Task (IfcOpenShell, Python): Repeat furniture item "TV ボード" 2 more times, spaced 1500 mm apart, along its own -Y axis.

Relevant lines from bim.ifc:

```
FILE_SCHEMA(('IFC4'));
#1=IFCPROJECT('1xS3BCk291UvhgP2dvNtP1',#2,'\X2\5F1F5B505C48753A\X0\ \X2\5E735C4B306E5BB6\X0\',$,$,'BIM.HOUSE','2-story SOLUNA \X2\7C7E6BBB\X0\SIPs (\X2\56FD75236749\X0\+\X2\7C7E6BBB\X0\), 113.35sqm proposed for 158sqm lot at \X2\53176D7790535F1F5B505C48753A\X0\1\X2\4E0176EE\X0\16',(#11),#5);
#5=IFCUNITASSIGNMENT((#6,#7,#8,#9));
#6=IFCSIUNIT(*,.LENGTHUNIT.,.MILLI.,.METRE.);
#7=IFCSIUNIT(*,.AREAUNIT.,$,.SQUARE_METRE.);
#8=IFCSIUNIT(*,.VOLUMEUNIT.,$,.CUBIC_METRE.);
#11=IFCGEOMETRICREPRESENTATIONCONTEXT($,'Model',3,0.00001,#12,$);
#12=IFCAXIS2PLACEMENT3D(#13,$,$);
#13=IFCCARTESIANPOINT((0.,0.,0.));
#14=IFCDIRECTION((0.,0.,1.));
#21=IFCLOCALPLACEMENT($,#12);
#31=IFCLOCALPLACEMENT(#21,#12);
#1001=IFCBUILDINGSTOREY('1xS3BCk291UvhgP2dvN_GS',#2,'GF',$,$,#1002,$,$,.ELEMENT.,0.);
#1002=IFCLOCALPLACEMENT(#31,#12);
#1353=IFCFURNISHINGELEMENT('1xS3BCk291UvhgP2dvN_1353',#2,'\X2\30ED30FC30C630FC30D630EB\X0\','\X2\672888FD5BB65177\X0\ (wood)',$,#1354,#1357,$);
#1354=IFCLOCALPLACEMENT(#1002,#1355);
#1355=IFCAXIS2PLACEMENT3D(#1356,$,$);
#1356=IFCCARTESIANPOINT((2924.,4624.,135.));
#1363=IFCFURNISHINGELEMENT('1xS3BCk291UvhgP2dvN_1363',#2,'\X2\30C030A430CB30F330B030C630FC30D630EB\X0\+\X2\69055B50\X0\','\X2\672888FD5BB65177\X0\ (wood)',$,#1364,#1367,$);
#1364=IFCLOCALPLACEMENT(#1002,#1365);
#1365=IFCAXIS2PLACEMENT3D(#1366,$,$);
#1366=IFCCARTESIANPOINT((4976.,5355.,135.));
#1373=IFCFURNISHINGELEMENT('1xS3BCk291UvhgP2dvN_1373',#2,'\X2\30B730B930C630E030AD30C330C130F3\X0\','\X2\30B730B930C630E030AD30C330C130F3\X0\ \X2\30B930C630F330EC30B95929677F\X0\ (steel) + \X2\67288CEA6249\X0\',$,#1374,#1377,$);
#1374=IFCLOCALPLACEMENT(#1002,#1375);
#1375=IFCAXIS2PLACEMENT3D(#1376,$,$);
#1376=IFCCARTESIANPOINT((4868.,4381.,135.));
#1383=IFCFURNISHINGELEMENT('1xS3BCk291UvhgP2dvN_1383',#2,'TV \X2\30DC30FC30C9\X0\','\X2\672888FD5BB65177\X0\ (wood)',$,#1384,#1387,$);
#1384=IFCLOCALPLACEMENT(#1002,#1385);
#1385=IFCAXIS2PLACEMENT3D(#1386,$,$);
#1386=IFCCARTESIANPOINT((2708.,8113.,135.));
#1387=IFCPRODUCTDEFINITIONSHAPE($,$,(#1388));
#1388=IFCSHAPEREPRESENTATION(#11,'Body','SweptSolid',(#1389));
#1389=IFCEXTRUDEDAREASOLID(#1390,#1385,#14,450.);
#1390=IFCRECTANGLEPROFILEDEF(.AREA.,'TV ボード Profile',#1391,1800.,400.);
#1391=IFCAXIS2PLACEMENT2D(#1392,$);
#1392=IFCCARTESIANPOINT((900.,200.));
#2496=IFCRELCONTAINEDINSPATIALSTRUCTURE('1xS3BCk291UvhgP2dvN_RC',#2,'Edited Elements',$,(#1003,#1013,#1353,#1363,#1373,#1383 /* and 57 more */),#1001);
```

```python
import ifcopenshell
import ifcopenshell.api.geometry
import ifcopenshell.api.root
import ifcopenshell.util.element
import ifcopenshell.util.placement

model = ifcopenshell.open("bim.ifc")


def reuse_history(source, copy):
    """copy_class also copies each property set's owner history, people and application; keep the originals."""
    for rel in copy.IsDefinedBy:
        if rel.is_a("IfcRelDefinesByProperties") and (history := rel.RelatingPropertyDefinition.OwnerHistory):
            rel.RelatingPropertyDefinition.OwnerHistory = source.OwnerHistory
            ifcopenshell.util.element.remove_deep2(model, history)


source = model.by_guid("1xS3BCk291UvhgP2dvN_1383")
base = ifcopenshell.util.placement.get_local_placement(source.ObjectPlacement)
step = -base[:3, 1] * 1500.0

for i in range(1, 3):
    copy = ifcopenshell.api.root.copy_class(model, product=source)
    copy.Representation = ifcopenshell.util.element.copy_deep(
        model, source.Representation, exclude=["IfcGeometricRepresentationContext", "IfcRepresentationMap"]
    )
    reuse_history(source, copy)
    matrix = base.copy()
    matrix[:3, 3] += i * step
    print("added at", matrix[:3, 3].round(3) + 0.0)
    ifcopenshell.api.geometry.edit_object_placement(model, product=copy, matrix=matrix, is_si=False)

model.write("bim_rev.ifc")
```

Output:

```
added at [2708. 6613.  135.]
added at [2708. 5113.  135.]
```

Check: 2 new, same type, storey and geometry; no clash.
